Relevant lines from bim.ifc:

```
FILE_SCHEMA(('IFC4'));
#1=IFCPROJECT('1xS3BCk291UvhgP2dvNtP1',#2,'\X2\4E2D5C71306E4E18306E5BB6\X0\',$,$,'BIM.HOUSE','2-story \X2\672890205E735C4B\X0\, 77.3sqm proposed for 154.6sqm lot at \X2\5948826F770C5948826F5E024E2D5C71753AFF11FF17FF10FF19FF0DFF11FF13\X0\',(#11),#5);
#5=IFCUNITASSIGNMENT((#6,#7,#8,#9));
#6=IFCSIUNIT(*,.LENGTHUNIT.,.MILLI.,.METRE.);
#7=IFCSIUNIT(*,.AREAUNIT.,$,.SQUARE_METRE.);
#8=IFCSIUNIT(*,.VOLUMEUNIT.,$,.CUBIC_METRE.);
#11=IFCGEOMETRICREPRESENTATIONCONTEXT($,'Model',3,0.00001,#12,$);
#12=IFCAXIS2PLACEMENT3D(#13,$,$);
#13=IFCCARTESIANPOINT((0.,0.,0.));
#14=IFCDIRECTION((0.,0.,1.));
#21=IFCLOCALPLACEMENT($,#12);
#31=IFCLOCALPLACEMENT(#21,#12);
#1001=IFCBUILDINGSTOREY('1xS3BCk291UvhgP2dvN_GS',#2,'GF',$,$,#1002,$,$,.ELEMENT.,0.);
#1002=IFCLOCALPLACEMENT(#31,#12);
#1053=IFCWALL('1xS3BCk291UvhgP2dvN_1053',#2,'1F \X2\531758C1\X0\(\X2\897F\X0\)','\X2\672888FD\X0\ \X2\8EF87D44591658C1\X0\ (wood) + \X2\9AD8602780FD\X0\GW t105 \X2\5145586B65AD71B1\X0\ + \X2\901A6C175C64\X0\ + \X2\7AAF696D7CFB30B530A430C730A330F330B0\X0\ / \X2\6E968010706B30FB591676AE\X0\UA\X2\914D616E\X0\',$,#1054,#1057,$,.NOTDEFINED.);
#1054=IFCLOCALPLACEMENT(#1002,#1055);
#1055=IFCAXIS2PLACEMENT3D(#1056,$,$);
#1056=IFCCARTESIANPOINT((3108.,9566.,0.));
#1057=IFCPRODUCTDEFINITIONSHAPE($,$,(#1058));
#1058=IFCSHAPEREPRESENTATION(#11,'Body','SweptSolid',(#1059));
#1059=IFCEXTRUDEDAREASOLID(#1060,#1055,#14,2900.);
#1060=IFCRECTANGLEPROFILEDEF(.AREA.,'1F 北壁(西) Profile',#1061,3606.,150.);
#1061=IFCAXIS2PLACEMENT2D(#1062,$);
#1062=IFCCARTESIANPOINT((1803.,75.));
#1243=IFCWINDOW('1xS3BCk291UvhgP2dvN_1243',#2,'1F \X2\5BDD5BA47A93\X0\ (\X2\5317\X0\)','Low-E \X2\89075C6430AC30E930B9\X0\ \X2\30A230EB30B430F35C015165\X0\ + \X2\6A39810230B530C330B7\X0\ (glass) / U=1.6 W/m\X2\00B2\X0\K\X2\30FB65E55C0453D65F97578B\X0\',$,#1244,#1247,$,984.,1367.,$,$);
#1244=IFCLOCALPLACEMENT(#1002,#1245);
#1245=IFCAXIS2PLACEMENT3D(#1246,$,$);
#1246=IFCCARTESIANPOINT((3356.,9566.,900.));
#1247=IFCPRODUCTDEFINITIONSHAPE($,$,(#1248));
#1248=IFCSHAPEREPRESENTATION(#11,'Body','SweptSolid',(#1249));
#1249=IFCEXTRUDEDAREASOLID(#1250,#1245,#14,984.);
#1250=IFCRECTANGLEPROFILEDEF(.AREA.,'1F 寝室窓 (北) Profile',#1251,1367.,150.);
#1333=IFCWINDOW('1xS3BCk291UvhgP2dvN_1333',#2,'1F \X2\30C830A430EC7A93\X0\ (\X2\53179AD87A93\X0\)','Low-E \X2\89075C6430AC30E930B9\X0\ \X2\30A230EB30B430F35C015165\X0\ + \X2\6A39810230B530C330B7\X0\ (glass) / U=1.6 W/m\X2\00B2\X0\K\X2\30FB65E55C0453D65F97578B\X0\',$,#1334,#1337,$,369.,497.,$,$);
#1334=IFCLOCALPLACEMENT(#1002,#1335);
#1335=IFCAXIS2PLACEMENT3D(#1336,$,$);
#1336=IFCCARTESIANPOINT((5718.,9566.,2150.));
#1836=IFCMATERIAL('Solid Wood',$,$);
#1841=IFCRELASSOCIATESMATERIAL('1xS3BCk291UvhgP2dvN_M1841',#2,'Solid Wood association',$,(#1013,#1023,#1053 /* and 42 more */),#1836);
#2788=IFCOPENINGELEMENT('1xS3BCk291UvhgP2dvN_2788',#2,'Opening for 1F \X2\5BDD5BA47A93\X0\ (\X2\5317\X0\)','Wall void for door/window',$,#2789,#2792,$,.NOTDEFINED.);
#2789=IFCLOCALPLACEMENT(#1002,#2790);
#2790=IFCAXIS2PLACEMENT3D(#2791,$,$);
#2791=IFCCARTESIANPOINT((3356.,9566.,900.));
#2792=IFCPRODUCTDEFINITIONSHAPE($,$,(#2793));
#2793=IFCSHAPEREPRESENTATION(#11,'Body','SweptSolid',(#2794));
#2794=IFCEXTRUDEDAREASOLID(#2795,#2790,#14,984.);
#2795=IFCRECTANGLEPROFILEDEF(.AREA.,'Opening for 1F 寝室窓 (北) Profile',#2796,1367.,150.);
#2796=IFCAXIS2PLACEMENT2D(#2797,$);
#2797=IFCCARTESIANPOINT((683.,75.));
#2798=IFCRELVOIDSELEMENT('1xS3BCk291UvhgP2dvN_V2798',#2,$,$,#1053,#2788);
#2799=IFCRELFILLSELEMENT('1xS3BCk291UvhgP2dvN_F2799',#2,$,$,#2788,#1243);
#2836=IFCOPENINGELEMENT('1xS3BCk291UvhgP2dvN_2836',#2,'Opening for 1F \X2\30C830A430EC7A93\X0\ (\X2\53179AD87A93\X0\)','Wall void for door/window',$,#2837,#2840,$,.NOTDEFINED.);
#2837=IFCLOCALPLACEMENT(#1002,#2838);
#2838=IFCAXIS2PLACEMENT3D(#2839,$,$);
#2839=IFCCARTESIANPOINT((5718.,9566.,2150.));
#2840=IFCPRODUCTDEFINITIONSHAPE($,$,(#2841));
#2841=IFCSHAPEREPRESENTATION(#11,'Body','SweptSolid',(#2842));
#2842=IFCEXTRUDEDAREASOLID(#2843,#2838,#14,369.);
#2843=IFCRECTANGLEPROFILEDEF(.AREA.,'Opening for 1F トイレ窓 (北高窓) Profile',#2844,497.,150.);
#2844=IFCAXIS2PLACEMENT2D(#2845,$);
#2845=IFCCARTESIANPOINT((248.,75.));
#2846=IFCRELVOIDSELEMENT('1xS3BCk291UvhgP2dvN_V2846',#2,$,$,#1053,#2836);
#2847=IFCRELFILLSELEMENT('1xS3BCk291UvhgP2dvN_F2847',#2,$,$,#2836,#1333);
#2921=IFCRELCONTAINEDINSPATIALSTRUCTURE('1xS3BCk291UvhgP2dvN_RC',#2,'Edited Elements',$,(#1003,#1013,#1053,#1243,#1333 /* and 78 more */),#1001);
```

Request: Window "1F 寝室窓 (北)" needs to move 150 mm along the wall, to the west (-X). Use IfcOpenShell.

```python
import ifcopenshell
import ifcopenshell.api.geometry
import ifcopenshell.util.placement

model = ifcopenshell.open("bim.ifc")

window = model.by_guid("1xS3BCk291UvhgP2dvN_1243")
opening = window.FillsVoids[0].RelatingOpeningElement
wall = opening.VoidsElements[0].RelatingBuildingElement

wall_matrix = ifcopenshell.util.placement.get_local_placement(wall.ObjectPlacement)
shift = wall_matrix[:3, 0] * -150.0
before = ifcopenshell.util.placement.get_local_placement(window.ObjectPlacement)[:3, 3].copy()

# The window is not placed relative to its opening, so move both.
for product in (opening, window):
    matrix = ifcopenshell.util.placement.get_local_placement(product.ObjectPlacement)
    matrix[:3, 3] += shift
    ifcopenshell.api.geometry.edit_object_placement(model, product=product, matrix=matrix, is_si=False)

after = ifcopenshell.util.placement.get_local_placement(window.ObjectPlacement)[:3, 3]
print("window moved by", (after - before).round(3) + 0.0)

model.write("bim_rev.ifc")
```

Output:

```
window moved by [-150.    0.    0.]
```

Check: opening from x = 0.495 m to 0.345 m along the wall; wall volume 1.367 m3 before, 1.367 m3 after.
